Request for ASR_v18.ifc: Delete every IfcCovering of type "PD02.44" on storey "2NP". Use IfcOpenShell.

First a look at what the model holds.

```python
import ifcopenshell
import ifcopenshell.util.element

model = ifcopenshell.open("ASR_v18.ifc")
print(model.schema)
storey = next(s for s in model.by_type("IfcBuildingStorey") if s.Name == "2NP")
coverings = [e for e in ifcopenshell.util.element.get_decomposition(storey) if e.is_a("IfcCovering")]
seen = {}
for e in coverings:
    element_type = ifcopenshell.util.element.get_type(e)
    name = element_type.Name if element_type not in (None, e) else None
    seen[name] = seen.get(name, 0) + 1
for name, count in sorted(seen.items(), key=str):
    print(count, "x", name)
```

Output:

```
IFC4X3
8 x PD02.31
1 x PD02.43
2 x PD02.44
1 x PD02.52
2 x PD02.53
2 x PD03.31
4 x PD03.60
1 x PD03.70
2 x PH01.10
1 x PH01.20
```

```python
import ifcopenshell
import ifcopenshell.api.root
import ifcopenshell.util.element

model = ifcopenshell.open("ASR_v18.ifc")

storey = next(s for s in model.by_type("IfcBuildingStorey") if s.Name == "2NP")
coverings = [e for e in ifcopenshell.util.element.get_decomposition(storey) if e.is_a("IfcCovering")]
targets = [e for e in coverings if (t := ifcopenshell.util.element.get_type(e)) not in (None, e) and t.Name == "PD02.44"]

for e in targets:
    ifcopenshell.api.root.remove_product(model, product=e)
print(len(targets), "removed")

model.write("ASR_v18_updated.ifc")
```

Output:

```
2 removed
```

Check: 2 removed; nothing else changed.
